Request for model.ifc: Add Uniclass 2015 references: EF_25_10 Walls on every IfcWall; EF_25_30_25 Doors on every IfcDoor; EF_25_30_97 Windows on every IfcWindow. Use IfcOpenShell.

First a look at what the model holds.

```python
import ifcopenshell

model = ifcopenshell.open("model.ifc")
print(model.schema)
print("classifications:", [c.Name for c in model.by_type("IfcClassification")])
for ifc_class in ("IfcDoor", "IfcRoof", "IfcStair", "IfcWall", "IfcWindow"):
    print(ifc_class, len(model.by_type(ifc_class)))
```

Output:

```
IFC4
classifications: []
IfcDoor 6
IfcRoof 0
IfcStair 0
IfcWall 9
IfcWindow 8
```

```python
import ifcopenshell
import ifcopenshell.api.classification

model = ifcopenshell.open("model.ifc")

system = ifcopenshell.api.classification.add_classification(model, classification="Uniclass 2015")

codes = {
    "IfcWall": ("EF_25_10", "Walls"),
    "IfcDoor": ("EF_25_30_25", "Doors"),
    "IfcWindow": ("EF_25_30_97", "Windows"),
}
for ifc_class, (code, name) in codes.items():
    products = model.by_type(ifc_class)
    ifcopenshell.api.classification.add_reference(
        model, products=products, classification=system, identification=code, name=name
    )
    print(code, len(products))

model.write("model_v2.ifc")
```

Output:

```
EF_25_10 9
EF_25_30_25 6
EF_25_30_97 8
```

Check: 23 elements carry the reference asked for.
